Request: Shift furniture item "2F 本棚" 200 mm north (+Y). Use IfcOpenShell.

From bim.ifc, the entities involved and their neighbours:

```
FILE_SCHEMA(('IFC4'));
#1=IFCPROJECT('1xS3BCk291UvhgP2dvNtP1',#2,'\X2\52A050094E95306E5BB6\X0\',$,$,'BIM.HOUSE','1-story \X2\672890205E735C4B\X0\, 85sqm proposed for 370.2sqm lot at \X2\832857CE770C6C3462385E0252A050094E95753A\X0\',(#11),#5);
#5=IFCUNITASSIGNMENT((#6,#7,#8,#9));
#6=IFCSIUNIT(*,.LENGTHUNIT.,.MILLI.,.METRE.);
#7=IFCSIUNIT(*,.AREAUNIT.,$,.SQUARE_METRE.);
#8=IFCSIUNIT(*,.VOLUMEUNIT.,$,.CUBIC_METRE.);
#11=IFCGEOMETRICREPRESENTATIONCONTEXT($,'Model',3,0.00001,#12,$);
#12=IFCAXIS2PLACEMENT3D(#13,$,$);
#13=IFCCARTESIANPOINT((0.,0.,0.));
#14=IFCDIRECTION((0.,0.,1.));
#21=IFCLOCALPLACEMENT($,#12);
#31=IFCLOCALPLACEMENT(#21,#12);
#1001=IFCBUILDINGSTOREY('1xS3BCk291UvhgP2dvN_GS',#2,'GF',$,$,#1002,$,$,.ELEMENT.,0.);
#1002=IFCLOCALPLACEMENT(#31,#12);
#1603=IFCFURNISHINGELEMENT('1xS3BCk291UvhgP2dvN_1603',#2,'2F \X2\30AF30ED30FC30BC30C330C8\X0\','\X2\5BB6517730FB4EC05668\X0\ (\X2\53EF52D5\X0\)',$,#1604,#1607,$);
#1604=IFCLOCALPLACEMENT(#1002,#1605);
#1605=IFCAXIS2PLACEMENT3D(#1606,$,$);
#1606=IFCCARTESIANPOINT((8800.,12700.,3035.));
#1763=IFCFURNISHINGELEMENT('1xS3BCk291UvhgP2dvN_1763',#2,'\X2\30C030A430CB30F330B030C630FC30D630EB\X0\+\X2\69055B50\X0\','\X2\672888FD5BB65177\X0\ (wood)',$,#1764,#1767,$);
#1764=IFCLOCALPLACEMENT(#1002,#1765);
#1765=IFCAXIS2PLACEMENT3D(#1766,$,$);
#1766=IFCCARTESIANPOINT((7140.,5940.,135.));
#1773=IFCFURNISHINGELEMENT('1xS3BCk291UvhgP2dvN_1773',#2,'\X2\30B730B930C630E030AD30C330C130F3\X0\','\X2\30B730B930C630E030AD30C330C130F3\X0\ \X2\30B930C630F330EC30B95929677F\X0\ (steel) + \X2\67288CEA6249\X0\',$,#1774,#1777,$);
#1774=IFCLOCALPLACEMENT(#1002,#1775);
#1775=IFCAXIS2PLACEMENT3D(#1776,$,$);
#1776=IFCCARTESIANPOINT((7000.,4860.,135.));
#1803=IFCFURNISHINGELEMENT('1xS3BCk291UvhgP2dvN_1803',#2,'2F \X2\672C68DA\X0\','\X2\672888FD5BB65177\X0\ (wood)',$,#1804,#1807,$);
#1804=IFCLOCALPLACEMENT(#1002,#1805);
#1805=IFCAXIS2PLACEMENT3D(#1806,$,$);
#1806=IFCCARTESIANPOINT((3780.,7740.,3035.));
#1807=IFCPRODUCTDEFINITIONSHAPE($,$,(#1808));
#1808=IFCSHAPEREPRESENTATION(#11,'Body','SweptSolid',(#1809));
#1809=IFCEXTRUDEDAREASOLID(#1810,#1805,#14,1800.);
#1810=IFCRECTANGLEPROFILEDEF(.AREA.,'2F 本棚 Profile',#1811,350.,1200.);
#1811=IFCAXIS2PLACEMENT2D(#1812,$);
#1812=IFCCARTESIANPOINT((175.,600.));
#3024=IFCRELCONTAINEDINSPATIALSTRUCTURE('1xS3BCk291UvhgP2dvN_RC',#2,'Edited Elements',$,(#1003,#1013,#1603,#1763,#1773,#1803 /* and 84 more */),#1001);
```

```python
import ifcopenshell
import ifcopenshell.api.geometry
import ifcopenshell.util.placement
import ifcopenshell.util.unit

model = ifcopenshell.open("bim.ifc")
unit_scale = ifcopenshell.util.unit.calculate_unit_scale(model)

item = model.by_guid("1xS3BCk291UvhgP2dvN_1803")
matrix = ifcopenshell.util.placement.get_local_placement(item.ObjectPlacement)
matrix[1, 3] += 0.2 / unit_scale
ifcopenshell.api.geometry.edit_object_placement(model, product=item, matrix=matrix, is_si=False)

print(ifcopenshell.util.placement.get_local_placement(item.ObjectPlacement).round(3) + 0.0)

model.write("bim_rev.ifc")
```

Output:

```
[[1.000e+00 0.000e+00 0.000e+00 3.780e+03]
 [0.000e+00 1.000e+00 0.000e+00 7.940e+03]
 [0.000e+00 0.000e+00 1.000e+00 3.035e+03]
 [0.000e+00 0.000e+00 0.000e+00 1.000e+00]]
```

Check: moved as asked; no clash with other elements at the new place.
